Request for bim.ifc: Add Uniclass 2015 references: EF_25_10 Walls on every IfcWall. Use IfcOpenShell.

First a look at what the model holds.

```python
import ifcopenshell

model = ifcopenshell.open("bim.ifc")
print(model.schema)
print("classifications:", [c.Name for c in model.by_type("IfcClassification")])
for ifc_class in ("IfcDoor", "IfcRoof", "IfcStair", "IfcWall", "IfcWindow"):
    print(ifc_class, len(model.by_type(ifc_class)))
```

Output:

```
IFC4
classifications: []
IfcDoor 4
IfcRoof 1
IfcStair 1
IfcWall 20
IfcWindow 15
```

```python
import ifcopenshell
import ifcopenshell.api.classification

model = ifcopenshell.open("bim.ifc")

system = ifcopenshell.api.classification.add_classification(model, classification="Uniclass 2015")

codes = {
    "IfcWall": ("EF_25_10", "Walls"),
}
for ifc_class, (code, name) in codes.items():
    products = model.by_type(ifc_class)
    ifcopenshell.api.classification.add_reference(
        model, products=products, classification=system, identification=code, name=name
    )
    print(code, len(products))

model.write("bim_updated.ifc")
```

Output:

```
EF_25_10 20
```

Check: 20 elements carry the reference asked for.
